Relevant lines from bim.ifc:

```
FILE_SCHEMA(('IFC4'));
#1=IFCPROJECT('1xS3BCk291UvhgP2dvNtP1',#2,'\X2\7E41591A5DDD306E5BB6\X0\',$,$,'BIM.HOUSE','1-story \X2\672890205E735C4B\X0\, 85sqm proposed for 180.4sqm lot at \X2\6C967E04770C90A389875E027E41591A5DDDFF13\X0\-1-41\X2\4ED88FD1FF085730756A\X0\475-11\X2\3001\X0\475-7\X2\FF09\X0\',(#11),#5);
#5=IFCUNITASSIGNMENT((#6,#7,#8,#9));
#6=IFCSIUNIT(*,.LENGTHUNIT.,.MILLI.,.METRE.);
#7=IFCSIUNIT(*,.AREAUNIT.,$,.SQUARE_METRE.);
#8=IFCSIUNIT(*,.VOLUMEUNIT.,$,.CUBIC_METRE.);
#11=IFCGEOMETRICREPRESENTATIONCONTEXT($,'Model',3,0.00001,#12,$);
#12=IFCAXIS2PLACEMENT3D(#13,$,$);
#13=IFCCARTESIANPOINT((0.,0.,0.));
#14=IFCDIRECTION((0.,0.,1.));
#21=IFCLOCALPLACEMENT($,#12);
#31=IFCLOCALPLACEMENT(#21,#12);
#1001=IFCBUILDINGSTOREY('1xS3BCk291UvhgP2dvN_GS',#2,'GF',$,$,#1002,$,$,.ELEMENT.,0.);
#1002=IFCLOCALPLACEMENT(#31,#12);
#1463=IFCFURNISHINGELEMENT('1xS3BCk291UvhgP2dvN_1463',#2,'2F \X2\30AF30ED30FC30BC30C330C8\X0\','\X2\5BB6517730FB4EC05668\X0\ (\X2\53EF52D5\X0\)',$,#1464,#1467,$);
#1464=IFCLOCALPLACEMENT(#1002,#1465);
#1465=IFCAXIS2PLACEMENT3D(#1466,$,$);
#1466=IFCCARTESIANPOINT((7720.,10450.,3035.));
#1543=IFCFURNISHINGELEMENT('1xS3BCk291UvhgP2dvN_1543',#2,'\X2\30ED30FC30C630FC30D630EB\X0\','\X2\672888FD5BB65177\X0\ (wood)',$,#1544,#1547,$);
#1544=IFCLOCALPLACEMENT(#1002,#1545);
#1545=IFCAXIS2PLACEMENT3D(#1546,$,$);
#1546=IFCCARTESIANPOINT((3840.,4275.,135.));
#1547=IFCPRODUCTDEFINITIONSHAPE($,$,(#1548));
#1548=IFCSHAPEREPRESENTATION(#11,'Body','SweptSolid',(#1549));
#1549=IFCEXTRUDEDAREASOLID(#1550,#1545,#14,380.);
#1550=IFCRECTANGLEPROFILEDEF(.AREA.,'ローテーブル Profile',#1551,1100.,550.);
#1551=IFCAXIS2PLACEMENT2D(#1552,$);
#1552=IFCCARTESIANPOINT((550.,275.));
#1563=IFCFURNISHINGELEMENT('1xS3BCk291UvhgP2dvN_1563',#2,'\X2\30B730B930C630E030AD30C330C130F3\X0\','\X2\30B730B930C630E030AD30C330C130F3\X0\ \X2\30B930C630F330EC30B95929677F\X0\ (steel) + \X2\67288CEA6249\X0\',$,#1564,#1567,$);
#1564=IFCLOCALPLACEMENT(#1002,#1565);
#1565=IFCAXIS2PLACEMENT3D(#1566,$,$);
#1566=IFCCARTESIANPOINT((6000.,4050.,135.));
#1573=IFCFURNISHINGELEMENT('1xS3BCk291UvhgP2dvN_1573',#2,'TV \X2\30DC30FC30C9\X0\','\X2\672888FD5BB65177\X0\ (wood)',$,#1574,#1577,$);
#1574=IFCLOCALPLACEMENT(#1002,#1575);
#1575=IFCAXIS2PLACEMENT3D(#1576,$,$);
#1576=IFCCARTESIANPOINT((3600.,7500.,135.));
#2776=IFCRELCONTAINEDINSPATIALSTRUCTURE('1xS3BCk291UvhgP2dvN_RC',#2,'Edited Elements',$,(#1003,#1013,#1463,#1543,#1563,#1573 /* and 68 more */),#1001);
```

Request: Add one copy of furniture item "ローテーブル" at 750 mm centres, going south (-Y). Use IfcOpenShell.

```python
import numpy as np
import ifcopenshell
import ifcopenshell.api.geometry
import ifcopenshell.api.root
import ifcopenshell.util.element
import ifcopenshell.util.placement

model = ifcopenshell.open("bim.ifc")


def reuse_history(source, copy):
    """copy_class also copies each property set's owner history, people and application; keep the originals."""
    for rel in copy.IsDefinedBy:
        if rel.is_a("IfcRelDefinesByProperties") and (history := rel.RelatingPropertyDefinition.OwnerHistory):
            rel.RelatingPropertyDefinition.OwnerHistory = source.OwnerHistory
            ifcopenshell.util.element.remove_deep2(model, history)


source = model.by_id(1543)
base = ifcopenshell.util.placement.get_local_placement(source.ObjectPlacement)
step = np.array([0.0, -1.0, 0.0]) * 750.0

for i in range(1, 2):
    copy = ifcopenshell.api.root.copy_class(model, product=source)
    copy.Representation = ifcopenshell.util.element.copy_deep(
        model, source.Representation, exclude=["IfcGeometricRepresentationContext", "IfcRepresentationMap"]
    )
    reuse_history(source, copy)
    matrix = base.copy()
    matrix[:3, 3] += i * step
    print("added at", matrix[:3, 3].round(3) + 0.0)
    ifcopenshell.api.geometry.edit_object_placement(model, product=copy, matrix=matrix, is_si=False)

model.write("bim_edited.ifc")
```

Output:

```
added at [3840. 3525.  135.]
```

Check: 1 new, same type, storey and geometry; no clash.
